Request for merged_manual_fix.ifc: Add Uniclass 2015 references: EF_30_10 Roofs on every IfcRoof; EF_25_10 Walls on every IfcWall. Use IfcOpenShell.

First a look at what the model holds.

```python
import ifcopenshell

model = ifcopenshell.open("merged_manual_fix.ifc")
print(model.schema)
print("classifications:", [c.Name for c in model.by_type("IfcClassification")])
for ifc_class in ("IfcDoor", "IfcRoof", "IfcStair", "IfcWall", "IfcWindow"):
    print(ifc_class, len(model.by_type(ifc_class)))
```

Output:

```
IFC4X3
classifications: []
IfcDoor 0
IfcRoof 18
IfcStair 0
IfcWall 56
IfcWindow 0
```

```python
import ifcopenshell
import ifcopenshell.api.classification

model = ifcopenshell.open("merged_manual_fix.ifc")

system = ifcopenshell.api.classification.add_classification(model, classification="Uniclass 2015")

codes = {
    "IfcRoof": ("EF_30_10", "Roofs"),
    "IfcWall": ("EF_25_10", "Walls"),
}
for ifc_class, (code, name) in codes.items():
    products = model.by_type(ifc_class)
    ifcopenshell.api.classification.add_reference(
        model, products=products, classification=system, identification=code, name=name
    )
    print(code, len(products))

model.write("merged_manual_fix_v2.ifc")
```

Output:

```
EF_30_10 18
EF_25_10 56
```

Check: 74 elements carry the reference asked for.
